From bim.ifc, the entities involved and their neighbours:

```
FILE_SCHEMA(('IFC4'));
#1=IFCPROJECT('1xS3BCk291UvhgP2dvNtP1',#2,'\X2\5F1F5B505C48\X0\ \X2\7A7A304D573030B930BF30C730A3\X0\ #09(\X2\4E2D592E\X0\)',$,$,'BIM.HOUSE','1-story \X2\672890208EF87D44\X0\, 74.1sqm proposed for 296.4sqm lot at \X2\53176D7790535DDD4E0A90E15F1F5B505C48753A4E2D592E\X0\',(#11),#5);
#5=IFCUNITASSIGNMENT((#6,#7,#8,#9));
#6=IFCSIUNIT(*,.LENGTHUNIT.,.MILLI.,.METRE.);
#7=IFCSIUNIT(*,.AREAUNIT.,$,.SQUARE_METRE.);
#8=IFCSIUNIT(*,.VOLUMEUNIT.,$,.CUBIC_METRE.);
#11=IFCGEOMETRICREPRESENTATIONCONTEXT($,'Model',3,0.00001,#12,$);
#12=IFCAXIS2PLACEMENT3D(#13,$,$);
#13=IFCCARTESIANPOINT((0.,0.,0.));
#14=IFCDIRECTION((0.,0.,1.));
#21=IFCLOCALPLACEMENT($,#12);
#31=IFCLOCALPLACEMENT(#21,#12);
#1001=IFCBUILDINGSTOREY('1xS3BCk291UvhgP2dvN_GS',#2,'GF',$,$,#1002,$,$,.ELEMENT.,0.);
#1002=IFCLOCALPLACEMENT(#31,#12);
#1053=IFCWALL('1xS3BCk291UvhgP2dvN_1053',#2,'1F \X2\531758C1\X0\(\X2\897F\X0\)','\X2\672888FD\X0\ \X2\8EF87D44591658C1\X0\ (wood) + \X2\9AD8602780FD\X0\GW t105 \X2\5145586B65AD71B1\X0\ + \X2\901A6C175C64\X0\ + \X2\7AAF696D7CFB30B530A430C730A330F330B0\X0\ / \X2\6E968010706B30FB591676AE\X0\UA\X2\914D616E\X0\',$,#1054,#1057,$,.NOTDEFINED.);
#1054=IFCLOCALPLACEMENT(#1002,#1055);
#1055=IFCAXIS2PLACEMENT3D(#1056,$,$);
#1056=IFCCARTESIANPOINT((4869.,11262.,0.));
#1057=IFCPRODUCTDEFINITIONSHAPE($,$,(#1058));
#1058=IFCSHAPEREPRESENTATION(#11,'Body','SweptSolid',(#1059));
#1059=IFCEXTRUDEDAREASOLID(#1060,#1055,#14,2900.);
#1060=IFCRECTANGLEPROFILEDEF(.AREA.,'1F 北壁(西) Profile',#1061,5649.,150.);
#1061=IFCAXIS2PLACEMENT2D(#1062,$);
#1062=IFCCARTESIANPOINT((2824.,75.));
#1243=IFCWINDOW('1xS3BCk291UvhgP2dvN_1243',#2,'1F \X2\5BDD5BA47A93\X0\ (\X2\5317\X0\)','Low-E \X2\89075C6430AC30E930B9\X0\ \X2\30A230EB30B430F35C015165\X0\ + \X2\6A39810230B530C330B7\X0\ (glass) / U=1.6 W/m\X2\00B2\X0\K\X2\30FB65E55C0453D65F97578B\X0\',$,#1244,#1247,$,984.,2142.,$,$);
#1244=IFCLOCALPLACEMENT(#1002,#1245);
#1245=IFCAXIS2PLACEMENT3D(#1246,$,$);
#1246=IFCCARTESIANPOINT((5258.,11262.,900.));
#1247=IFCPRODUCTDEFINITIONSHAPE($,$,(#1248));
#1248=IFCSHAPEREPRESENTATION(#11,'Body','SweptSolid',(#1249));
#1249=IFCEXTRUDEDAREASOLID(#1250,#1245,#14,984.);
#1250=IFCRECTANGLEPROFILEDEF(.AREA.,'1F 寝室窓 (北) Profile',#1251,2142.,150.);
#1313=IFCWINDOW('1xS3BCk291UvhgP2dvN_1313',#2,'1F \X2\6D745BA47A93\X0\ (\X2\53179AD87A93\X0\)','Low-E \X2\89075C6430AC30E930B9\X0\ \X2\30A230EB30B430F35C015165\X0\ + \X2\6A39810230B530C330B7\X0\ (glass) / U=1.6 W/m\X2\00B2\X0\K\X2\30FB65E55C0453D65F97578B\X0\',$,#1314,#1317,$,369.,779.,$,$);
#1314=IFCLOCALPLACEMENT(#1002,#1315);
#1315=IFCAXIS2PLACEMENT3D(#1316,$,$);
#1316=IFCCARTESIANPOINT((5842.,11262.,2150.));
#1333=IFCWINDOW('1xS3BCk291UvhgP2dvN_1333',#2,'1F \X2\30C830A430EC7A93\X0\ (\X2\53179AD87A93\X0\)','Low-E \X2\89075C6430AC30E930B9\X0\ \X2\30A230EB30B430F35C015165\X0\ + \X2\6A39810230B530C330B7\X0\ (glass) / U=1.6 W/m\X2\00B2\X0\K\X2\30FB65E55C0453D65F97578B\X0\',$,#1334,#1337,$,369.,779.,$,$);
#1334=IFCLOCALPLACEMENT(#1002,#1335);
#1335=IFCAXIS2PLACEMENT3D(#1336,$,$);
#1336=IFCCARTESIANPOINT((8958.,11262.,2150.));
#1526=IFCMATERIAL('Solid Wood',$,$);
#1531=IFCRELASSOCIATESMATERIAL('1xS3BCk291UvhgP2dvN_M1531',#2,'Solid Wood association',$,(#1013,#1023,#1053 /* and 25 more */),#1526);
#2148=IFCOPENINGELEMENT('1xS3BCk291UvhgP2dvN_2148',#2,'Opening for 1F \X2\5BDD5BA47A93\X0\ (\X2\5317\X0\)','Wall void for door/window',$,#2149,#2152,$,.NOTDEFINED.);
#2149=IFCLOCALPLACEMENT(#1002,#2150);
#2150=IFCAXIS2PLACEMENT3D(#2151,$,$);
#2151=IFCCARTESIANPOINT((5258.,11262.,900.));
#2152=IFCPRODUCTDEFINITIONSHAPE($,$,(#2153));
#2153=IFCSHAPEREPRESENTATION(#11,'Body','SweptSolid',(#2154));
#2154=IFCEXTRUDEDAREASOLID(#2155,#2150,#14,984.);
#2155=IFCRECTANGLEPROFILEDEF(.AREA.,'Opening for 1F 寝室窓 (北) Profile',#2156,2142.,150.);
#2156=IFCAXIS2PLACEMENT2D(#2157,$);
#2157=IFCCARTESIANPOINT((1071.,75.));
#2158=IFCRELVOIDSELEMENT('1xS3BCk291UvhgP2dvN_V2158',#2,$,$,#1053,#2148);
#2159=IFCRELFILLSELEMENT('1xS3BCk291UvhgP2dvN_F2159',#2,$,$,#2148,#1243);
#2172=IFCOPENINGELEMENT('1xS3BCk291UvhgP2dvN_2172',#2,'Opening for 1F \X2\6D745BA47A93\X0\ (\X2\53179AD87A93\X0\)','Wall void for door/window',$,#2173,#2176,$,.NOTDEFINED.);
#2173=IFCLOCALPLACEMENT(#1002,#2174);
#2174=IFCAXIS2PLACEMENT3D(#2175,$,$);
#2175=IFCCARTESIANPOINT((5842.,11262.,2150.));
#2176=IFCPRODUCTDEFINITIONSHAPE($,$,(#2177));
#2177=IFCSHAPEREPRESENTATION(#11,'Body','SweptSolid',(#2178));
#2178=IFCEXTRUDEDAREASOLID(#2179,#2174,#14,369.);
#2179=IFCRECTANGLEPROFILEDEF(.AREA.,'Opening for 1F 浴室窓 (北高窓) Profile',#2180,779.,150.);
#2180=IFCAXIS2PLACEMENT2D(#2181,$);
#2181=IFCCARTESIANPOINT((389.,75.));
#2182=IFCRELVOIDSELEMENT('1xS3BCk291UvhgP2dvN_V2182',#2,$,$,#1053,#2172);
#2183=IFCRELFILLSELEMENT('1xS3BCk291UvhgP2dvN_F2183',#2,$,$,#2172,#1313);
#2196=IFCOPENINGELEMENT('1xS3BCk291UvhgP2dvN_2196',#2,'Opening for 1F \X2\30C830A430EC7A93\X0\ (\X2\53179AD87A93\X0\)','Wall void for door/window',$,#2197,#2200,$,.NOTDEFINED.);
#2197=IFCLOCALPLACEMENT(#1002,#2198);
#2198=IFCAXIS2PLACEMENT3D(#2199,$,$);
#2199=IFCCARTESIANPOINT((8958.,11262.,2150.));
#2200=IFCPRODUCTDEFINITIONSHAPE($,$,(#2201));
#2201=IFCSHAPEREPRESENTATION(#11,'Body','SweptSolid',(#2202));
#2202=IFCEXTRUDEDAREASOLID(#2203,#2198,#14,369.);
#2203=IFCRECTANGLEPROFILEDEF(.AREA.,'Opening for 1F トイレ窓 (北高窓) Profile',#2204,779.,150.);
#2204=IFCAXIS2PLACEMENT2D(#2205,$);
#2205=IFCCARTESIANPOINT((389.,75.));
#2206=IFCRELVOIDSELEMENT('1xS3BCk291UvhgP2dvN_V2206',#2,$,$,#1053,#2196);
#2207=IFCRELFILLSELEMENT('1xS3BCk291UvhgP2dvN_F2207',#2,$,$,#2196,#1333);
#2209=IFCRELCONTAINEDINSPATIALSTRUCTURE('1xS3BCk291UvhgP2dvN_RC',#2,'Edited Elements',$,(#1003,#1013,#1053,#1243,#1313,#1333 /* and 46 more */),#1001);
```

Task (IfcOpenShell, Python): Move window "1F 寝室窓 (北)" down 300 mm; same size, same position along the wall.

```python
import numpy as np
import ifcopenshell
import ifcopenshell.api.geometry
import ifcopenshell.util.placement
import ifcopenshell.util.unit

model = ifcopenshell.open("bim.ifc")
unit_scale = ifcopenshell.util.unit.calculate_unit_scale(model)

window = model.by_guid("1xS3BCk291UvhgP2dvN_1243")
opening = window.FillsVoids[0].RelatingOpeningElement
dz = -300.0

shift = np.array([0.0, 0.0, dz])
# The window is not placed relative to its opening, so move both.
for product in (opening, window):
    matrix = ifcopenshell.util.placement.get_local_placement(product.ObjectPlacement)
    matrix[:3, 3] += shift
    ifcopenshell.api.geometry.edit_object_placement(model, product=product, matrix=matrix, is_si=False)

print(f"moved by {dz * unit_scale:+.3f} m")

model.write("bim_updated.ifc")
```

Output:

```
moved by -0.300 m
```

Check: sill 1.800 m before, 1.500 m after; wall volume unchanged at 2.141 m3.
